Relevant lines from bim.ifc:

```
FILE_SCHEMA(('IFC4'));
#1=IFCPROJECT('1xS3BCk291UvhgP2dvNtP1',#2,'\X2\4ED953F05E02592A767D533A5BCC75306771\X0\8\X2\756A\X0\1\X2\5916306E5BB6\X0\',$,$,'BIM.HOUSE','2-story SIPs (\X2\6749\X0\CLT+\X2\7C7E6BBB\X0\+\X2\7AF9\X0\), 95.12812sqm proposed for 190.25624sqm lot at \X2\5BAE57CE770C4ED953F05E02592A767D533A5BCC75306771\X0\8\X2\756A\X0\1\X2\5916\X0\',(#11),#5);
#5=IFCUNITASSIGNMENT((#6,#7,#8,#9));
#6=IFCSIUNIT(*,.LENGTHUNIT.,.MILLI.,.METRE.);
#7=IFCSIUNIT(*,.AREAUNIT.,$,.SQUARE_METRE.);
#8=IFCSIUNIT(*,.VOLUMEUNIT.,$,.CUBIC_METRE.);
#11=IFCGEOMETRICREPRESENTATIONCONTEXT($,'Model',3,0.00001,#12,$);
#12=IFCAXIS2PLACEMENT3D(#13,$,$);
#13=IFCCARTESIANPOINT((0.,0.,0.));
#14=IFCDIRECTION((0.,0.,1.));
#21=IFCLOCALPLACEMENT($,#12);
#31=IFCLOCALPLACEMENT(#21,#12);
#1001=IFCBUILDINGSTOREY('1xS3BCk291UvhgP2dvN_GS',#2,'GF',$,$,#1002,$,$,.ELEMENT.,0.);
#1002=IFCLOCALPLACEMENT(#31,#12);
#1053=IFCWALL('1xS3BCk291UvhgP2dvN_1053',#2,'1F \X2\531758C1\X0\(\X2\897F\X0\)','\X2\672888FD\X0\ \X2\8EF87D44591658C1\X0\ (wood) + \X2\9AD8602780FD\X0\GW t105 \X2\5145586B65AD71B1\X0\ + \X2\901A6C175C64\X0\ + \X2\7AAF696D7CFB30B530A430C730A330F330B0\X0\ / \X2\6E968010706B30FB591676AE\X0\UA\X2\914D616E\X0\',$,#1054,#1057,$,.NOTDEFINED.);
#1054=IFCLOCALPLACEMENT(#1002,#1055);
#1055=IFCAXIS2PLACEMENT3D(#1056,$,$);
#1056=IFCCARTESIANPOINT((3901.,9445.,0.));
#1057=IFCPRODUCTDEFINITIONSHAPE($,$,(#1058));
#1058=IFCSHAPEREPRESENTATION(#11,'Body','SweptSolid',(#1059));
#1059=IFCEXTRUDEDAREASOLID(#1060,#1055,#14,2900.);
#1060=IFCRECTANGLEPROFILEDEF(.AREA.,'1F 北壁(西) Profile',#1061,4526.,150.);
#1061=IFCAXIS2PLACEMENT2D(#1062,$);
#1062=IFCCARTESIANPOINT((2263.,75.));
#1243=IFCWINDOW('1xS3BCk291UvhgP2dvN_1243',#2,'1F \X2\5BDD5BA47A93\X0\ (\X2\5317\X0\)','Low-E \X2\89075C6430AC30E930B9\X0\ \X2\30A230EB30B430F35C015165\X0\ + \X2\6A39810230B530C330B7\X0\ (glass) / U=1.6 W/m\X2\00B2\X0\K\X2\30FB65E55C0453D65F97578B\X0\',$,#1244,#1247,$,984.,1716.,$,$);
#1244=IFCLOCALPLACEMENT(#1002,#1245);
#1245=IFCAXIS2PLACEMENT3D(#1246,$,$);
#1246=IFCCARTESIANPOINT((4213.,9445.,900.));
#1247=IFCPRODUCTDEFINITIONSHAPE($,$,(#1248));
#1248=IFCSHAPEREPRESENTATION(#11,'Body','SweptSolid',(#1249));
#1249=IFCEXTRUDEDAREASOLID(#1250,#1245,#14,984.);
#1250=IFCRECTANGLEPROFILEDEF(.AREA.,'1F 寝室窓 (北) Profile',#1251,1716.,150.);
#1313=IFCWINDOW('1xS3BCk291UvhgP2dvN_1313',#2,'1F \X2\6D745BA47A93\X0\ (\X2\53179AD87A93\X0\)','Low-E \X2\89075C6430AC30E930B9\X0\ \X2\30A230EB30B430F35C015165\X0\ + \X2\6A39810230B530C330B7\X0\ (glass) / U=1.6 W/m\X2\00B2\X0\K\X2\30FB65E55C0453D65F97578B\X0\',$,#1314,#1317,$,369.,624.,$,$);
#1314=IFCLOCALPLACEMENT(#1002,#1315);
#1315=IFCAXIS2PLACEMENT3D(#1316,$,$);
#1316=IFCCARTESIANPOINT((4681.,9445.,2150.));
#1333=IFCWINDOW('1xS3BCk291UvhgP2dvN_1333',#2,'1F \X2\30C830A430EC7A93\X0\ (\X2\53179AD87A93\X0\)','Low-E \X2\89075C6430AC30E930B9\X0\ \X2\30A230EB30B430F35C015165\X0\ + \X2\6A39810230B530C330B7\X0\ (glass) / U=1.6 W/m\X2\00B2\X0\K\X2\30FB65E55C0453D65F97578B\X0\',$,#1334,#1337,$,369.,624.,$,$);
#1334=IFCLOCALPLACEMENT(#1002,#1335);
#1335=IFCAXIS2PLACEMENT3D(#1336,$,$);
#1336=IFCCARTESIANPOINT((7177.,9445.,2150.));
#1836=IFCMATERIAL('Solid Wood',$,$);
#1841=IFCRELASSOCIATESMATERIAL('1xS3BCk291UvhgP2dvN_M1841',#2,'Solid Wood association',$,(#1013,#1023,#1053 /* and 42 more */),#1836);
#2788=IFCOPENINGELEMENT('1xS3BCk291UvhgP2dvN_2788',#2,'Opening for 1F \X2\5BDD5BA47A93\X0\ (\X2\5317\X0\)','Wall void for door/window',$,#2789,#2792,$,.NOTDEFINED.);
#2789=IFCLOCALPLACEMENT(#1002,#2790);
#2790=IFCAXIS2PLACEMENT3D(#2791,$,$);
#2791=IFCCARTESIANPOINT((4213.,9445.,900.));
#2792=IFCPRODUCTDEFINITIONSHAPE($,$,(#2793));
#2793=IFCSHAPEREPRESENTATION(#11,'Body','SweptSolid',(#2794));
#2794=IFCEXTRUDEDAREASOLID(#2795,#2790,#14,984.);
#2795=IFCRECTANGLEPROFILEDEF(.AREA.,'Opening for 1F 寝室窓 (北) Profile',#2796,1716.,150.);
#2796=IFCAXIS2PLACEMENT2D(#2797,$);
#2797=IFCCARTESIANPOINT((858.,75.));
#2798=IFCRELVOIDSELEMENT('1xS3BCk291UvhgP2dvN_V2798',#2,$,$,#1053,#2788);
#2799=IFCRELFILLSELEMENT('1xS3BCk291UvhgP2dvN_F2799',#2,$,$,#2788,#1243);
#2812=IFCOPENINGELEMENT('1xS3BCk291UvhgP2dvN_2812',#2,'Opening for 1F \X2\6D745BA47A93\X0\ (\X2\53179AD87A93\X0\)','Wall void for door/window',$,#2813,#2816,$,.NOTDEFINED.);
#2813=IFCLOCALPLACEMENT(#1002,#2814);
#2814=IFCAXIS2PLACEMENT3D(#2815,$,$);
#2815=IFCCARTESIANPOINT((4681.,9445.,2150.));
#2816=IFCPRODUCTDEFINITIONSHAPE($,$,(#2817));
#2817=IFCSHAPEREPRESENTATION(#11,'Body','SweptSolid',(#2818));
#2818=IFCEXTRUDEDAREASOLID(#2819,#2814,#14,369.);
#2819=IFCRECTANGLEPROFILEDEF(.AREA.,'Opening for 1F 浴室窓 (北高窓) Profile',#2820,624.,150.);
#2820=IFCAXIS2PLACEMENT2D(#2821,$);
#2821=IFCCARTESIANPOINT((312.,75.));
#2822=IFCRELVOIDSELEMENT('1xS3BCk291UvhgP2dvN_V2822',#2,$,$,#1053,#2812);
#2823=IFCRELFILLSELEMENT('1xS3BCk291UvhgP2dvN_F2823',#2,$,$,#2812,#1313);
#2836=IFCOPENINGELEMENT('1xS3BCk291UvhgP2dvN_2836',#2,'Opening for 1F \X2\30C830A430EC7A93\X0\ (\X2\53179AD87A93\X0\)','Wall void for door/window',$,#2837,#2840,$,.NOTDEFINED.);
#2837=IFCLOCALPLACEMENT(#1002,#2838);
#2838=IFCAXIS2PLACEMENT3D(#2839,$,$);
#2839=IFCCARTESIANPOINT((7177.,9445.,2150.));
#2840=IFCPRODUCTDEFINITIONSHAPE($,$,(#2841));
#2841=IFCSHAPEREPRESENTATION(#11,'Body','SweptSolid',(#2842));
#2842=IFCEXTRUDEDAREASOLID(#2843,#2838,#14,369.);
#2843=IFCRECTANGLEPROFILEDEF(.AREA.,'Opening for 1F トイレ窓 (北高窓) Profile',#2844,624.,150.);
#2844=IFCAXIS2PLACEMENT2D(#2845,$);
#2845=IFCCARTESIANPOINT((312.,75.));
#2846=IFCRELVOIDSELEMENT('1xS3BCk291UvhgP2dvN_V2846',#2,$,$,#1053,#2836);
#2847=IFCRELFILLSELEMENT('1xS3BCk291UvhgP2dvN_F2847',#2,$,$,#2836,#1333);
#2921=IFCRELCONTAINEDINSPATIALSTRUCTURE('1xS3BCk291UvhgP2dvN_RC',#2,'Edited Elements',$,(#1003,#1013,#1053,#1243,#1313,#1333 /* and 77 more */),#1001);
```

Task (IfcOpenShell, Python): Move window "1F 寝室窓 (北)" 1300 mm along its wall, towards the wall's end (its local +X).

```python
import ifcopenshell
import ifcopenshell.api.geometry
import ifcopenshell.util.placement

model = ifcopenshell.open("bim.ifc")

window = model.by_id(1243)
opening = window.FillsVoids[0].RelatingOpeningElement
wall = opening.VoidsElements[0].RelatingBuildingElement

wall_matrix = ifcopenshell.util.placement.get_local_placement(wall.ObjectPlacement)
shift = wall_matrix[:3, 0] * 1300.0
before = ifcopenshell.util.placement.get_local_placement(window.ObjectPlacement)[:3, 3].copy()

# The window is not placed relative to its opening, so move both.
for product in (opening, window):
    matrix = ifcopenshell.util.placement.get_local_placement(product.ObjectPlacement)
    matrix[:3, 3] += shift
    ifcopenshell.api.geometry.edit_object_placement(model, product=product, matrix=matrix, is_si=False)

after = ifcopenshell.util.placement.get_local_placement(window.ObjectPlacement)[:3, 3]
print("window moved by", (after - before).round(3) + 0.0)

model.write("bim_updated.ifc")
```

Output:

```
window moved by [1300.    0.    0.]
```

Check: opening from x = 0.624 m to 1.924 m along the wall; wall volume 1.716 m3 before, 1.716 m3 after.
